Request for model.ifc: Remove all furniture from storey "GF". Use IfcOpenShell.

First a look at what the model holds.

```python
import ifcopenshell
import ifcopenshell.util.element

model = ifcopenshell.open("model.ifc")
print(model.schema)
storey = next(s for s in model.by_type("IfcBuildingStorey") if s.Name == "GF")
furniture = [e for e in ifcopenshell.util.element.get_decomposition(storey) if e.is_a("IfcFurnishingElement")]
seen = {}
for e in furniture:
    element_type = ifcopenshell.util.element.get_type(e)
    name = element_type.Name if element_type not in (None, e) else None
    seen[name] = seen.get(name, 0) + 1
for name, count in sorted(seen.items(), key=str):
    print(count, "x", name)
```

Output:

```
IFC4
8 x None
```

```python
import ifcopenshell
import ifcopenshell.api.root
import ifcopenshell.util.element

model = ifcopenshell.open("model.ifc")

storey = next(s for s in model.by_type("IfcBuildingStorey") if s.Name == "GF")
furniture = [e for e in ifcopenshell.util.element.get_decomposition(storey) if e.is_a("IfcFurnishingElement")]

for e in furniture:
    ifcopenshell.api.root.remove_product(model, product=e)
print(len(furniture), "removed")

model.write("model-out.ifc")
```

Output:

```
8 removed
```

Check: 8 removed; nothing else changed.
